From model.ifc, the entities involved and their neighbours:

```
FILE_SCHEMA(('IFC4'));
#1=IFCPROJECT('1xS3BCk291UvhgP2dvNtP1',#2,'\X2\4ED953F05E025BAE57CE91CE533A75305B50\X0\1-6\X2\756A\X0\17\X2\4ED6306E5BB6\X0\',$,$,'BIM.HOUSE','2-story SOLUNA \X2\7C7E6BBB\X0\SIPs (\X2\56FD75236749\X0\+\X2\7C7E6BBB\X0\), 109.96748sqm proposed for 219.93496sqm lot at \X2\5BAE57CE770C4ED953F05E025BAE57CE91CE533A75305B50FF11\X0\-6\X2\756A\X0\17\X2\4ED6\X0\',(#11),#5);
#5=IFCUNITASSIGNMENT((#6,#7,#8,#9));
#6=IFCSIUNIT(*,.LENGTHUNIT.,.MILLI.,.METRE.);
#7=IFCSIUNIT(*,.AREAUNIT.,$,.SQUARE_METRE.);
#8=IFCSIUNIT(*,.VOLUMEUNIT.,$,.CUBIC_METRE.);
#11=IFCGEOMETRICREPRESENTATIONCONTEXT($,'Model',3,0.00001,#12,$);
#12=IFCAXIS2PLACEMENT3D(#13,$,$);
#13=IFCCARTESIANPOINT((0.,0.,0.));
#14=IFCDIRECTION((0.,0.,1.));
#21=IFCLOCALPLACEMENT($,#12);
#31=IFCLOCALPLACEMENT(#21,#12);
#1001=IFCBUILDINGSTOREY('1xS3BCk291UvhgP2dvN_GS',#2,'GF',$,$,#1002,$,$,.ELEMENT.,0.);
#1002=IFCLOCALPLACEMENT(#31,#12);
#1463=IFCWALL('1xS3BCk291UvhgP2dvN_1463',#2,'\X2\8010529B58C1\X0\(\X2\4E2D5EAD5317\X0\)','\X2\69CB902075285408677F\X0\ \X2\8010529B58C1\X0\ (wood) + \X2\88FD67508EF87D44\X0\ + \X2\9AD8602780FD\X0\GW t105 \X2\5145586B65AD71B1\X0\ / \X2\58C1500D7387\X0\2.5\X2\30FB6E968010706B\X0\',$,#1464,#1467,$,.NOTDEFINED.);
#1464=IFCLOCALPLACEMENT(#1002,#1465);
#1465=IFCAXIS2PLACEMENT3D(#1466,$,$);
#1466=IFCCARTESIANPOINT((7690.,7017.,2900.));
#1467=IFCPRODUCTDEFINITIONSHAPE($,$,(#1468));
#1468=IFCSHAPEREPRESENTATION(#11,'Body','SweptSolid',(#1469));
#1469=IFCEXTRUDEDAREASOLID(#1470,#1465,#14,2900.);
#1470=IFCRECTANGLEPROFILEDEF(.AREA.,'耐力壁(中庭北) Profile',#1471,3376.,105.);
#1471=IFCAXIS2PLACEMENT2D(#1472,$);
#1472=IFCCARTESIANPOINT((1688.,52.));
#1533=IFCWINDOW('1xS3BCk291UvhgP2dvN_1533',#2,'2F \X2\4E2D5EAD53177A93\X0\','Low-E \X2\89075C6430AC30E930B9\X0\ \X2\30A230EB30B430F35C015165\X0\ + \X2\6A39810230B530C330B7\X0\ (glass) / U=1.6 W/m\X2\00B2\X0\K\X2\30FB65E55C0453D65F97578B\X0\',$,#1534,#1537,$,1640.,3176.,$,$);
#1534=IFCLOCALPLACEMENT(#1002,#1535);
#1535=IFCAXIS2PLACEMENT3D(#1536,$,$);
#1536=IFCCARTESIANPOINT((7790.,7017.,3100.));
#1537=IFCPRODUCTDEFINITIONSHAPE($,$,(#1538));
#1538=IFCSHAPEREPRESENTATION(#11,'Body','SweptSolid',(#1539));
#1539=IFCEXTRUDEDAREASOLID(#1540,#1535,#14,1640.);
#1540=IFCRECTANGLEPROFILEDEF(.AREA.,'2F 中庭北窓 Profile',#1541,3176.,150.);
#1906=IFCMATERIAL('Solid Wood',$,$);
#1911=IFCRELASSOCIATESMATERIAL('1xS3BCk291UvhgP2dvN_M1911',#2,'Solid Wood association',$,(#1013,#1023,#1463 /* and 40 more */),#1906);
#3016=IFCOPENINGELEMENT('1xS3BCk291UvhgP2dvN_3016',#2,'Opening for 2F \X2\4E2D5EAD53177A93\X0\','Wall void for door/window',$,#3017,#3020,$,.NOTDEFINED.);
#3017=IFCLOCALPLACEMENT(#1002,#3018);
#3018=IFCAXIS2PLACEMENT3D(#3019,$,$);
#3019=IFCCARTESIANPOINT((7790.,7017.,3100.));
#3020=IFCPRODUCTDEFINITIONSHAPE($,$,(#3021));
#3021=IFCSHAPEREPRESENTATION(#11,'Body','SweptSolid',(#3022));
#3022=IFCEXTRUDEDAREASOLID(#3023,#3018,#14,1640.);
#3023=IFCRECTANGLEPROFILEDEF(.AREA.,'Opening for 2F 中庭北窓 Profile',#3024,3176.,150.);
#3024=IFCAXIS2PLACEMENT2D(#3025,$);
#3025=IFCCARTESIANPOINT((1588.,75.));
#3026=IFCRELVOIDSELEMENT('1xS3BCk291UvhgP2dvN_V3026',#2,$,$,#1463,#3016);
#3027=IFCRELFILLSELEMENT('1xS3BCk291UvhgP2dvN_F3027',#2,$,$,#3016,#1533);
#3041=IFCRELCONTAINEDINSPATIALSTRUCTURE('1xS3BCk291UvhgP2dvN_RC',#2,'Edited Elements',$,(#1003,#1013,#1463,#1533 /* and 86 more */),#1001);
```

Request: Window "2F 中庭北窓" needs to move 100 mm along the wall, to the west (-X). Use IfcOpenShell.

```python
import ifcopenshell
import ifcopenshell.api.geometry
import ifcopenshell.util.placement
import ifcopenshell.util.unit

model = ifcopenshell.open("model.ifc")
unit_scale = ifcopenshell.util.unit.calculate_unit_scale(model)

window = model.by_id(1533)
opening = window.FillsVoids[0].RelatingOpeningElement
wall = opening.VoidsElements[0].RelatingBuildingElement

wall_matrix = ifcopenshell.util.placement.get_local_placement(wall.ObjectPlacement)
shift = wall_matrix[:3, 0] * -0.1 / unit_scale
before = ifcopenshell.util.placement.get_local_placement(window.ObjectPlacement)[:3, 3].copy()

# The window is not placed relative to its opening, so move both.
for product in (opening, window):
    matrix = ifcopenshell.util.placement.get_local_placement(product.ObjectPlacement)
    matrix[:3, 3] += shift
    ifcopenshell.api.geometry.edit_object_placement(model, product=product, matrix=matrix, is_si=False)

after = ifcopenshell.util.placement.get_local_placement(window.ObjectPlacement)[:3, 3]
print("window moved by", (after - before).round(3) + 0.0)

model.write("model_v2.ifc")
```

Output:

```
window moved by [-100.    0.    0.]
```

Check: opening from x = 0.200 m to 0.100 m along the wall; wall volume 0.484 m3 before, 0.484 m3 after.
